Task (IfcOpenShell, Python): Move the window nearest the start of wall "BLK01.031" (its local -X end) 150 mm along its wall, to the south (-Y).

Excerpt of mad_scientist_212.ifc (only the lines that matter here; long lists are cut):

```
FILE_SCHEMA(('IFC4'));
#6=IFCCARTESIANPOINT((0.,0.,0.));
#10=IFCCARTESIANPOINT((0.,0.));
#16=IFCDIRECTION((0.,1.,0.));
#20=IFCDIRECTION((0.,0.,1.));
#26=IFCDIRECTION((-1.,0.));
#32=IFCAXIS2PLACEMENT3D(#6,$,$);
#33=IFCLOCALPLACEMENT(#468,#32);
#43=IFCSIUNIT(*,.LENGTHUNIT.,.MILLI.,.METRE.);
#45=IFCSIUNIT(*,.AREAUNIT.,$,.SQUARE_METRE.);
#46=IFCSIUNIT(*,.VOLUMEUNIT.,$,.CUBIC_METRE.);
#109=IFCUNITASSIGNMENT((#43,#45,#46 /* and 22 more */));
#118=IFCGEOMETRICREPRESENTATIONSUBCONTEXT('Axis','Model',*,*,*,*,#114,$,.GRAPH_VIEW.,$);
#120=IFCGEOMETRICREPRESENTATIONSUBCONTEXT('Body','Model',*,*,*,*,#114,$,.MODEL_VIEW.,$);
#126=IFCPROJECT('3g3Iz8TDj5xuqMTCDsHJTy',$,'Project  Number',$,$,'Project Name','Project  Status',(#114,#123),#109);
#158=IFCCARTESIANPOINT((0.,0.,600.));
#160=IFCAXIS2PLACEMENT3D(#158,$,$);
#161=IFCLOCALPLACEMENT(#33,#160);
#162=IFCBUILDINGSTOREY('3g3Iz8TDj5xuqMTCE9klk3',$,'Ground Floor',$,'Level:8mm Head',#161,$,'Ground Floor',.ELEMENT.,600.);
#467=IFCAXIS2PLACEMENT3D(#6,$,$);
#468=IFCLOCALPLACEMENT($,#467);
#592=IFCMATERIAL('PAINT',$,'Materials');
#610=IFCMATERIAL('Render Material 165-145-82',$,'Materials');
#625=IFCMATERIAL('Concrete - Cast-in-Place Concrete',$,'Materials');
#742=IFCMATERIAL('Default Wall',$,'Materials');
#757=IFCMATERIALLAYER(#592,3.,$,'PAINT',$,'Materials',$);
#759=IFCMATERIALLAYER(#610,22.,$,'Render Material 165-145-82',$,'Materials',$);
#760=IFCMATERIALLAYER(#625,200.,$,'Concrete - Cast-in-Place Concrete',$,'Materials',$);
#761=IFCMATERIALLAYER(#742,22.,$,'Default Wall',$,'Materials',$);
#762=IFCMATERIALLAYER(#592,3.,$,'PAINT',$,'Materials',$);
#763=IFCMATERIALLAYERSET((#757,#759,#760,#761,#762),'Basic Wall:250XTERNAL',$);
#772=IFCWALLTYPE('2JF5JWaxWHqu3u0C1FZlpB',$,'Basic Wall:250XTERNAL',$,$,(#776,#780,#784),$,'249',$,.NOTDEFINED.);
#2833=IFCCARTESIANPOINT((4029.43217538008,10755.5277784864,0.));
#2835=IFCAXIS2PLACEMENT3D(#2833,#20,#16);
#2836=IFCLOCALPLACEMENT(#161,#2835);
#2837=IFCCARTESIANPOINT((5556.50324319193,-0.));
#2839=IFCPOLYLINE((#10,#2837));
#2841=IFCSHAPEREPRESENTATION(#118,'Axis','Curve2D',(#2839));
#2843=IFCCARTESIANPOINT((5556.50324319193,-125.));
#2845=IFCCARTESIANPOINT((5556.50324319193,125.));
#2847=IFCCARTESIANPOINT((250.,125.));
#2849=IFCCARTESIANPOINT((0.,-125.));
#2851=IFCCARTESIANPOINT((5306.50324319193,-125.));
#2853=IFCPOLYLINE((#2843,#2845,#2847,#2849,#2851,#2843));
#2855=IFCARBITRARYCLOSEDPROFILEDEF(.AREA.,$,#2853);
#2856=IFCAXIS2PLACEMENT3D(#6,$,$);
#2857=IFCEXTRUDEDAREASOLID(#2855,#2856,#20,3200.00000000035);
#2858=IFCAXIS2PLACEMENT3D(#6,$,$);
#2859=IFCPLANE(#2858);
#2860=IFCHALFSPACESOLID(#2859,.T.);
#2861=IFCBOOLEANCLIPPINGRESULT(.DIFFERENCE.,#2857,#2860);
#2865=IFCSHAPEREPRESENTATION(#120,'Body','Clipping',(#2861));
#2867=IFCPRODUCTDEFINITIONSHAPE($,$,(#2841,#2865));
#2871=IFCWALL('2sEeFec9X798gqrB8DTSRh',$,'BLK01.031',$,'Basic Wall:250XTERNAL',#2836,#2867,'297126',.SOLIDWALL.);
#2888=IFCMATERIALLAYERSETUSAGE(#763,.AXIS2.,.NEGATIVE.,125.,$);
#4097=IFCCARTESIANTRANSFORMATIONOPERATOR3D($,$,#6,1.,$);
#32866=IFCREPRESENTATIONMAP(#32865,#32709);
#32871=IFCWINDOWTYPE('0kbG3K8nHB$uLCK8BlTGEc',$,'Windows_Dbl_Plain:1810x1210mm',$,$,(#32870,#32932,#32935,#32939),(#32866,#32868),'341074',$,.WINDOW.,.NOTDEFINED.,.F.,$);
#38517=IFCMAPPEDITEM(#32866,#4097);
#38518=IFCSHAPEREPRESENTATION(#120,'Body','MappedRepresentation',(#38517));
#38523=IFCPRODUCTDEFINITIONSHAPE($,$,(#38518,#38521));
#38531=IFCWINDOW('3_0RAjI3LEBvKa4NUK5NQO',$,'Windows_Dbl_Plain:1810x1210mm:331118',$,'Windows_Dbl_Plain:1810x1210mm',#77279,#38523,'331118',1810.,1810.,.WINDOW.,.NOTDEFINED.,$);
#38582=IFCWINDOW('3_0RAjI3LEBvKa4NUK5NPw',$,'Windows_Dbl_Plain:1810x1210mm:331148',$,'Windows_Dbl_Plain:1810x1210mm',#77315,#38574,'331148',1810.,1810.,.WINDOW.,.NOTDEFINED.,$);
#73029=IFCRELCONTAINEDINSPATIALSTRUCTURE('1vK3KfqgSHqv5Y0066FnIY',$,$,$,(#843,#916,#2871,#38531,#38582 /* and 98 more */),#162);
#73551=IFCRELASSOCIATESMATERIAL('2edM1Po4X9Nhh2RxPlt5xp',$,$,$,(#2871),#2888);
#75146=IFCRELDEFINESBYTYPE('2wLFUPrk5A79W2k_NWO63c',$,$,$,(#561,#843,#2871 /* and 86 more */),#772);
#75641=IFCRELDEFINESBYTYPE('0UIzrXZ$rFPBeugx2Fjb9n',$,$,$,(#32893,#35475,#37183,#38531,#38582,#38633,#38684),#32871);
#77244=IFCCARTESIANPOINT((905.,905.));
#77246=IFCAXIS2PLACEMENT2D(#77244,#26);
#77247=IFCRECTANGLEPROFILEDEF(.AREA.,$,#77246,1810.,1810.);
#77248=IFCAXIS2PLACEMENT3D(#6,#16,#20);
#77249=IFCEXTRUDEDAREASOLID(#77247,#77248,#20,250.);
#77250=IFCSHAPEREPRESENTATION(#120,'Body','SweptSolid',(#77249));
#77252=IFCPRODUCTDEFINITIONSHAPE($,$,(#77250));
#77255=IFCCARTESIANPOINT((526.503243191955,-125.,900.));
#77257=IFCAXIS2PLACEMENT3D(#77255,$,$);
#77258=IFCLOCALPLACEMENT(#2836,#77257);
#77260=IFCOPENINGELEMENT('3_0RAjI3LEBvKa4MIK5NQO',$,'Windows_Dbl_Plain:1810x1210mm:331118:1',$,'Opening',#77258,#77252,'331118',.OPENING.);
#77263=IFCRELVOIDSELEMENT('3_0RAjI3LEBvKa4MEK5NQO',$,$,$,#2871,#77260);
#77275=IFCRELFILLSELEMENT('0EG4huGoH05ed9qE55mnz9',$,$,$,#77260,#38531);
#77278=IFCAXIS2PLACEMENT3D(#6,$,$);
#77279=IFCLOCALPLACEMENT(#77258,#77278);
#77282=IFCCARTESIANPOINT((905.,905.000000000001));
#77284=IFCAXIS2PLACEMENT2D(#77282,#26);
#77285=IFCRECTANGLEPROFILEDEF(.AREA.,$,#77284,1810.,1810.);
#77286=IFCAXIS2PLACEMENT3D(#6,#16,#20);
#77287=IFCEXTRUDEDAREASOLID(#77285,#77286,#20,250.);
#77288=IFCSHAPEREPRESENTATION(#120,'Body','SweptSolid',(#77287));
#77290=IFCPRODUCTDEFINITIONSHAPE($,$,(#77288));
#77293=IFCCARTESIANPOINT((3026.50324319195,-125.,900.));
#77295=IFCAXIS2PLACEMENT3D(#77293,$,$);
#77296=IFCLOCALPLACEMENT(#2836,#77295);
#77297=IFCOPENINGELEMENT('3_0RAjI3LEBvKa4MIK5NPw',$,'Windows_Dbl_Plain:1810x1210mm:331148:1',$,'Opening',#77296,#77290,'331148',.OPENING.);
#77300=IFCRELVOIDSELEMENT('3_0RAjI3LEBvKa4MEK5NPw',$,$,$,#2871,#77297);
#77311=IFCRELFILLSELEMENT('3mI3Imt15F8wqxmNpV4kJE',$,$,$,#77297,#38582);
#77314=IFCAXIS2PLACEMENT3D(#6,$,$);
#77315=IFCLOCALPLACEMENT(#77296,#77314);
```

```python
import ifcopenshell
import ifcopenshell.api.geometry
import ifcopenshell.util.placement
import ifcopenshell.util.unit

model = ifcopenshell.open("mad_scientist_212.ifc")
unit_scale = ifcopenshell.util.unit.calculate_unit_scale(model)

window = model.by_id(38531)
opening = window.FillsVoids[0].RelatingOpeningElement
wall = opening.VoidsElements[0].RelatingBuildingElement

wall_matrix = ifcopenshell.util.placement.get_local_placement(wall.ObjectPlacement)
shift = wall_matrix[:3, 0] * -0.15 / unit_scale
before = ifcopenshell.util.placement.get_local_placement(window.ObjectPlacement)[:3, 3].copy()

# The window is placed relative to its opening, so it follows when the opening moves.
matrix = ifcopenshell.util.placement.get_local_placement(opening.ObjectPlacement)
matrix[:3, 3] += shift
ifcopenshell.api.geometry.edit_object_placement(
    model, product=opening, matrix=matrix, is_si=False, should_transform_children=True
)

after = ifcopenshell.util.placement.get_local_placement(window.ObjectPlacement)[:3, 3]
print("window moved by", (after - before).round(3) + 0.0)

model.write("mad_scientist_212_updated.ifc")
```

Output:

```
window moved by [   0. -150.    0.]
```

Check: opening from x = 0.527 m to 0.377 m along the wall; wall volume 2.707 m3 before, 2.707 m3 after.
